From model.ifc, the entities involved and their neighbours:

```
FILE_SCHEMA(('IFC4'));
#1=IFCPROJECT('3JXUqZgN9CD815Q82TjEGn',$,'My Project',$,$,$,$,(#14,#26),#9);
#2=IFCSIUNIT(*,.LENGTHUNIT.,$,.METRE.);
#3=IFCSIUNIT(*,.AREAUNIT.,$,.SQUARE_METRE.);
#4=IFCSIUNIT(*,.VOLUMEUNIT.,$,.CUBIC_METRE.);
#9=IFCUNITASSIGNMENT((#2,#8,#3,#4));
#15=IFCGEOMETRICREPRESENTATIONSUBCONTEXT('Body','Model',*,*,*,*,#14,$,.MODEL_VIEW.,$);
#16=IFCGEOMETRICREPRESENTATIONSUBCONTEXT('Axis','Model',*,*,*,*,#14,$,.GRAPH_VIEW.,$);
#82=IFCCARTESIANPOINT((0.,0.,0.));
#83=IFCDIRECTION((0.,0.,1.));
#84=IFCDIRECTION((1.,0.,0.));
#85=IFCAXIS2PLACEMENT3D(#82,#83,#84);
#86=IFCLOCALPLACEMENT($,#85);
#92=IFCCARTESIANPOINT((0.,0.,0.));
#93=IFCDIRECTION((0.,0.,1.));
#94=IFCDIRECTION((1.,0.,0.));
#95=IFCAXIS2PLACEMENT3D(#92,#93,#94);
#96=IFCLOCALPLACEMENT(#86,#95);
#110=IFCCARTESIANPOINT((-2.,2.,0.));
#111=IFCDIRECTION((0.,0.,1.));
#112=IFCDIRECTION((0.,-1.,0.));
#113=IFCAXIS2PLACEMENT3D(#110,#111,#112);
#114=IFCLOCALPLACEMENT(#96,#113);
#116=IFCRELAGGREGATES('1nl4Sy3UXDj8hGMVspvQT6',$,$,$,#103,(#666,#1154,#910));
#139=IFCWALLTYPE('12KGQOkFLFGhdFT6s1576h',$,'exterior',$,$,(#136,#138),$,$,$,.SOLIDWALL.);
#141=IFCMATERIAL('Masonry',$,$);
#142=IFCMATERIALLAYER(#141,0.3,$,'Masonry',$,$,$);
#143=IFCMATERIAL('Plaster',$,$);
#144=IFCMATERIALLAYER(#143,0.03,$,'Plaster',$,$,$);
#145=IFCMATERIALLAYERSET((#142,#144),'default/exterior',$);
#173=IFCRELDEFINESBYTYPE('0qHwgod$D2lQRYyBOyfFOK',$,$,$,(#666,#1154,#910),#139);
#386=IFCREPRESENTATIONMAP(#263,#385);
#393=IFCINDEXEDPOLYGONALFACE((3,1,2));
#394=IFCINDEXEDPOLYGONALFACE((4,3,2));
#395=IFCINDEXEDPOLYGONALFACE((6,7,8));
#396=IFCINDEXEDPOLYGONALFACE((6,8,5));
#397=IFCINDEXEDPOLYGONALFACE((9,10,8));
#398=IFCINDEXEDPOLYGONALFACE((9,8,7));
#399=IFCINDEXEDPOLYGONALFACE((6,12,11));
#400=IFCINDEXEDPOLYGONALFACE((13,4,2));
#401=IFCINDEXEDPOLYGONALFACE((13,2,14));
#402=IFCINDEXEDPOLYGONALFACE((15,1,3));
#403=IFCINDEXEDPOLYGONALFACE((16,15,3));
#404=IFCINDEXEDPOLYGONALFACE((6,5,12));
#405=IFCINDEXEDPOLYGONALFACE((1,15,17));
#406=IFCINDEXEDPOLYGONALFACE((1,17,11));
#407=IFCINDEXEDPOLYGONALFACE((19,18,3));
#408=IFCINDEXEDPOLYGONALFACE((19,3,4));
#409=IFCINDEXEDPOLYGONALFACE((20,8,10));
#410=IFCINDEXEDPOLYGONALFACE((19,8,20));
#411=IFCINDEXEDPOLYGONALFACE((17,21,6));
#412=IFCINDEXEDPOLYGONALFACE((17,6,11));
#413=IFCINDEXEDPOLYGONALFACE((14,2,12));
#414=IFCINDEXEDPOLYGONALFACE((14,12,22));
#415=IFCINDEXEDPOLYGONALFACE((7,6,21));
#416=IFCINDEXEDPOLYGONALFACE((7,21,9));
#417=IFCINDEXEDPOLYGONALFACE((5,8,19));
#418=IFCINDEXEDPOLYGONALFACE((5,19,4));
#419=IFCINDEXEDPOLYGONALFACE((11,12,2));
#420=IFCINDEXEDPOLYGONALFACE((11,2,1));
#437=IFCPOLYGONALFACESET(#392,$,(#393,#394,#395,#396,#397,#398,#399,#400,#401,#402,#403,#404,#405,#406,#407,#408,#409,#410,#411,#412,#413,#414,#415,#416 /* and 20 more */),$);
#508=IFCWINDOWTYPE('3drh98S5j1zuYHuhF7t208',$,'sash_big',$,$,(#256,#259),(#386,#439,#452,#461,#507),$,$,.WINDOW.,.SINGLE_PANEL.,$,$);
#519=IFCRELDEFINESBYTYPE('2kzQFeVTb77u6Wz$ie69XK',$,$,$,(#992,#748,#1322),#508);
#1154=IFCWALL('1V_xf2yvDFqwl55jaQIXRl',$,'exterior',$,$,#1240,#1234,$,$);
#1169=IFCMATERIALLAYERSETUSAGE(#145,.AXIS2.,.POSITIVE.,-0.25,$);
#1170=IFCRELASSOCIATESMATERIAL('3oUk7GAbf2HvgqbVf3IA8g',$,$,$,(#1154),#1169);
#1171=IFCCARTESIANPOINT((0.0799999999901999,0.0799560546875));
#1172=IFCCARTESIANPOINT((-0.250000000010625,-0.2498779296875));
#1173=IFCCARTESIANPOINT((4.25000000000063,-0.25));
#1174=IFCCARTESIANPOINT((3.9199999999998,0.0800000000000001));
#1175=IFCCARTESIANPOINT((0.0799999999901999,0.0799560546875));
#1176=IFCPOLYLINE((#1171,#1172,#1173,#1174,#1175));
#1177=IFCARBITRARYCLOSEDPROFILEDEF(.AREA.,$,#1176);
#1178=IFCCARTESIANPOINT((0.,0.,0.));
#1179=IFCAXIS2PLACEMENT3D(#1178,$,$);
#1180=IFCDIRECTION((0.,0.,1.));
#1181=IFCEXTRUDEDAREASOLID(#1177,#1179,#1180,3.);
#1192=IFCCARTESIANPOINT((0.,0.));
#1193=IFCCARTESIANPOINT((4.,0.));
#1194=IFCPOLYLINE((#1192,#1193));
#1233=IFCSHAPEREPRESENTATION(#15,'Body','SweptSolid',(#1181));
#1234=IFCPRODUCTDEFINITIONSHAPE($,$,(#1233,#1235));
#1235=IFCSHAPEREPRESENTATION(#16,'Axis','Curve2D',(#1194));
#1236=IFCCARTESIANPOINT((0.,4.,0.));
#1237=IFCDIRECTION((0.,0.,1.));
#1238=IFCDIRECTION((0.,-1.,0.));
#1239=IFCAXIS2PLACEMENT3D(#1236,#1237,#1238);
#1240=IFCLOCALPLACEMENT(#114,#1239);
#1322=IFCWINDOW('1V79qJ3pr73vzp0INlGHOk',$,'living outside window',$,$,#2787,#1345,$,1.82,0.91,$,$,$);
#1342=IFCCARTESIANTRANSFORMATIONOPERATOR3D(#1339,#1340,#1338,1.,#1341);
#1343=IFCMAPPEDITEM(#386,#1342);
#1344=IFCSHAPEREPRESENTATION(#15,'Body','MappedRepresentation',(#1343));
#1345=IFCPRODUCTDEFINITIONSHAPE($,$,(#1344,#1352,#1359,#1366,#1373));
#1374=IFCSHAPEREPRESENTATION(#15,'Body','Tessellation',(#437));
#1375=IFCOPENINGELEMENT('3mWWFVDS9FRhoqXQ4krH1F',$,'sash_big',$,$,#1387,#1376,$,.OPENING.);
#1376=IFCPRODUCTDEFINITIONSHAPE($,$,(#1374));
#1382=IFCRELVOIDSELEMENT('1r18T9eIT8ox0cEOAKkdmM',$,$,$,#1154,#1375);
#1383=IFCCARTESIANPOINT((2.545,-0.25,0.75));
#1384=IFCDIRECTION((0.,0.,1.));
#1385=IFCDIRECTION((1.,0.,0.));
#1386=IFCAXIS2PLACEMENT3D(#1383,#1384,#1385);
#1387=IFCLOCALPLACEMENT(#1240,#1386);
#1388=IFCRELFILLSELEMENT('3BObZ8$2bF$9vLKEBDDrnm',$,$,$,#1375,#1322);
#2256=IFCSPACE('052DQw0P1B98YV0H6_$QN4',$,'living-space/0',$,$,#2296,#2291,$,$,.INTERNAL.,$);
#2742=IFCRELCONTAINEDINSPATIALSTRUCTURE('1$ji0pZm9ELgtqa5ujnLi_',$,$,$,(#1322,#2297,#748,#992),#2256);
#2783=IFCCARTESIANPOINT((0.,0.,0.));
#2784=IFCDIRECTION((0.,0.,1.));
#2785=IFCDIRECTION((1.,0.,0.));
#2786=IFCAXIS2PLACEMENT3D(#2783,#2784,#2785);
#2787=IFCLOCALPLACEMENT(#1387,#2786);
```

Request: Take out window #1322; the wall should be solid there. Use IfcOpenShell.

```python
import ifcopenshell
import ifcopenshell.api.feature
import ifcopenshell.api.root
import ifcopenshell.geom
import ifcopenshell.util.shape

model = ifcopenshell.open("model.ifc")
settings = ifcopenshell.geom.settings()


def volume(element):
    """Net volume in cubic metres, openings subtracted."""
    shape = ifcopenshell.geom.create_shape(settings, element)
    return ifcopenshell.util.shape.get_volume(shape.geometry)


window = model.by_guid("1V79qJ3pr73vzp0INlGHOk")
opening = window.FillsVoids[0].RelatingOpeningElement
wall = opening.VoidsElements[0].RelatingBuildingElement
before = volume(wall)

ifcopenshell.api.root.remove_product(model, product=window)
ifcopenshell.api.feature.remove_feature(model, feature=opening)

after = volume(wall)

print(f"wall volume {before:.3f} -> {after:.3f} m3")

model.write("model_edited.ifc")
```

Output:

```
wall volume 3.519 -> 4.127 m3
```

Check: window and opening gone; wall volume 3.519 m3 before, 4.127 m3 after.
